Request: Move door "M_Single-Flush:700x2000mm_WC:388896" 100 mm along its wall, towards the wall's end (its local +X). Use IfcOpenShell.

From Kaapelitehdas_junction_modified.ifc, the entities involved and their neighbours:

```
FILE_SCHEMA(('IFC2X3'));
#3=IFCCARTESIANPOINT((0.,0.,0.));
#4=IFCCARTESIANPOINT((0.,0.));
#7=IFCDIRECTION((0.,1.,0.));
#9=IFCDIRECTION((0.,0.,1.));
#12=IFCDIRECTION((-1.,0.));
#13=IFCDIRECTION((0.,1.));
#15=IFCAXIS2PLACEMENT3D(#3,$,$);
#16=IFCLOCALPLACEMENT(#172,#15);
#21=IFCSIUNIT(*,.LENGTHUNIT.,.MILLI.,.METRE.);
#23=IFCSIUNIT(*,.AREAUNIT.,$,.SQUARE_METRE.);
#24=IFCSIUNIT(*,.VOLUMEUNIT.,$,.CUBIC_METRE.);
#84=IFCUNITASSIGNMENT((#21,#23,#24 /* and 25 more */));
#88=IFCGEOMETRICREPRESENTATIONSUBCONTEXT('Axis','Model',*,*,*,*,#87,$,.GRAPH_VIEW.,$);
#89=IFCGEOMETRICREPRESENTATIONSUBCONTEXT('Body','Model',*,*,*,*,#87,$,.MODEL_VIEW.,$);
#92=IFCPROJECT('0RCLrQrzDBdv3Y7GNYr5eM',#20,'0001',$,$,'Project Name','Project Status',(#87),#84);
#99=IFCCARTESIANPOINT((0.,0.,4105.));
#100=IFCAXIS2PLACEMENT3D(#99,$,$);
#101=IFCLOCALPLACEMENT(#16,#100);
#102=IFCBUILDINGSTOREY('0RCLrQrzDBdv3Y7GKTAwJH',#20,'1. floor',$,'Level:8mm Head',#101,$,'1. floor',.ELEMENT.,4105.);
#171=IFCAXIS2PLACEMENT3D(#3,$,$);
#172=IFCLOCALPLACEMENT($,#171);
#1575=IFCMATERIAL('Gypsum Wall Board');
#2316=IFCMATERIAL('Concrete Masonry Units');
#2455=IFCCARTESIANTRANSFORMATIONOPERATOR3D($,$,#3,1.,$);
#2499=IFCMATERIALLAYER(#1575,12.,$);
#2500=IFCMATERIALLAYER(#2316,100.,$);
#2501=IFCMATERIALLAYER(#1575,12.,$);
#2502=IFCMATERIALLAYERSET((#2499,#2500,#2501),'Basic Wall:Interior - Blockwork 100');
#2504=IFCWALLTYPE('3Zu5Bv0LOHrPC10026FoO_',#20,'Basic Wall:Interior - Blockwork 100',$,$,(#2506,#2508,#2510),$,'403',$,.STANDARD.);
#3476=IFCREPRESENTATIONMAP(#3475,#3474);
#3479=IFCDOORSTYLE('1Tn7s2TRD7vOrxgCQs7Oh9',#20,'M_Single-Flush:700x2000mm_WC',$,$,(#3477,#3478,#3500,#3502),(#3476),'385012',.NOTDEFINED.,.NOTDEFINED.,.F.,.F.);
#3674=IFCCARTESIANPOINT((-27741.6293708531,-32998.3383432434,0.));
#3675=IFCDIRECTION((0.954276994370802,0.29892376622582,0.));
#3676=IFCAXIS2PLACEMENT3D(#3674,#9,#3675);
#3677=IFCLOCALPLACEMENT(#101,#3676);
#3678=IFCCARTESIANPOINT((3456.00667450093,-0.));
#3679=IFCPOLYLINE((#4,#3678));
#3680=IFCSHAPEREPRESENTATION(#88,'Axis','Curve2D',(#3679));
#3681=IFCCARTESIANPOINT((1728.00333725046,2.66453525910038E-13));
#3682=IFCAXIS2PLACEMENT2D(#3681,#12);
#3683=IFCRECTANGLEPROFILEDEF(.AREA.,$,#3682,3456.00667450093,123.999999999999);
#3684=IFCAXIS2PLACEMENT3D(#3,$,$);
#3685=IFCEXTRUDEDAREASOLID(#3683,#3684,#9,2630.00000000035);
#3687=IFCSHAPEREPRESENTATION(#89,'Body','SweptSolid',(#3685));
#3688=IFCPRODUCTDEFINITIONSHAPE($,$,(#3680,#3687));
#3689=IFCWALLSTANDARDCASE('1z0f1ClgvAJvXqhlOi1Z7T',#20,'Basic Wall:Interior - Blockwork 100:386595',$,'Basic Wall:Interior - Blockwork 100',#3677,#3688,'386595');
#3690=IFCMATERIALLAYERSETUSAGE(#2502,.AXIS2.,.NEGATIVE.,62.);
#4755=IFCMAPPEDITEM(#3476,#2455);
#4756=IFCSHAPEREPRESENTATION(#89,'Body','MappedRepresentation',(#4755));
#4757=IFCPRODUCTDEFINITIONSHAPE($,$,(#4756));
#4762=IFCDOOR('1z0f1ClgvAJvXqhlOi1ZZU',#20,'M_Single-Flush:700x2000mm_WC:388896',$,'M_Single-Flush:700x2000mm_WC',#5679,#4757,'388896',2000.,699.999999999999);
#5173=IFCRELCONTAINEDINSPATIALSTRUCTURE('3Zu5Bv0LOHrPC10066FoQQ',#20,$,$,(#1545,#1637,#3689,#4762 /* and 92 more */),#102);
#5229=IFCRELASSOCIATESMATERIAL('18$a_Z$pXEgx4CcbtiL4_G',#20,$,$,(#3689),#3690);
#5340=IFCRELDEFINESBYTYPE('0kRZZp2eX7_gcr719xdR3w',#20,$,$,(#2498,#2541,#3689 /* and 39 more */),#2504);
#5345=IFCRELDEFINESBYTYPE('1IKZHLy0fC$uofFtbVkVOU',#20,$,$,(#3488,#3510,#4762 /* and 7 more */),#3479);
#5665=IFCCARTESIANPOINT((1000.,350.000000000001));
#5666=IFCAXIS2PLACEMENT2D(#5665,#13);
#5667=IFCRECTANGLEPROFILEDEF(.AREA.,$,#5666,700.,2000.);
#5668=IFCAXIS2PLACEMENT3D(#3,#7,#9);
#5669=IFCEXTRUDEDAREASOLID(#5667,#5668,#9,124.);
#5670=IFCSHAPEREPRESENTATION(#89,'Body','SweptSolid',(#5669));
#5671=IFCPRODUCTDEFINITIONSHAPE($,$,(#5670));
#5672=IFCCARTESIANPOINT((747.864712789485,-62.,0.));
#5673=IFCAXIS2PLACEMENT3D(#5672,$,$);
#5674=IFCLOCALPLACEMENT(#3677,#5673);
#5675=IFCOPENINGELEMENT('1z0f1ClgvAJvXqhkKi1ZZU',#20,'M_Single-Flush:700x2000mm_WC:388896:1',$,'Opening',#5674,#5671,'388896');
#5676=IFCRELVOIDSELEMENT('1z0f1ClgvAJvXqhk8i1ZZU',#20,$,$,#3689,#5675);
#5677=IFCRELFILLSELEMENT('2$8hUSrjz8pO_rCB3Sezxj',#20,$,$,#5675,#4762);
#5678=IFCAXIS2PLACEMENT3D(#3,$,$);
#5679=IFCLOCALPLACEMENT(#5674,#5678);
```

```python
import ifcopenshell
import ifcopenshell.api.geometry
import ifcopenshell.util.placement

model = ifcopenshell.open("Kaapelitehdas_junction_modified.ifc")

door = model.by_id(4762)
opening = door.FillsVoids[0].RelatingOpeningElement
wall = opening.VoidsElements[0].RelatingBuildingElement

wall_matrix = ifcopenshell.util.placement.get_local_placement(wall.ObjectPlacement)
shift = wall_matrix[:3, 0] * 100.0
before = ifcopenshell.util.placement.get_local_placement(door.ObjectPlacement)[:3, 3].copy()

# The door is placed relative to its opening, so it follows when the opening moves.
matrix = ifcopenshell.util.placement.get_local_placement(opening.ObjectPlacement)
matrix[:3, 3] += shift
ifcopenshell.api.geometry.edit_object_placement(
    model, product=opening, matrix=matrix, is_si=False, should_transform_children=True
)

after = ifcopenshell.util.placement.get_local_placement(door.ObjectPlacement)[:3, 3]
print("door moved by", (after - before).round(3) + 0.0)

model.write("Kaapelitehdas_junction_modified_edited.ifc")
```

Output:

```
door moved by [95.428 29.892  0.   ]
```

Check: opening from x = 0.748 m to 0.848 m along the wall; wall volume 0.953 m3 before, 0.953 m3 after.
